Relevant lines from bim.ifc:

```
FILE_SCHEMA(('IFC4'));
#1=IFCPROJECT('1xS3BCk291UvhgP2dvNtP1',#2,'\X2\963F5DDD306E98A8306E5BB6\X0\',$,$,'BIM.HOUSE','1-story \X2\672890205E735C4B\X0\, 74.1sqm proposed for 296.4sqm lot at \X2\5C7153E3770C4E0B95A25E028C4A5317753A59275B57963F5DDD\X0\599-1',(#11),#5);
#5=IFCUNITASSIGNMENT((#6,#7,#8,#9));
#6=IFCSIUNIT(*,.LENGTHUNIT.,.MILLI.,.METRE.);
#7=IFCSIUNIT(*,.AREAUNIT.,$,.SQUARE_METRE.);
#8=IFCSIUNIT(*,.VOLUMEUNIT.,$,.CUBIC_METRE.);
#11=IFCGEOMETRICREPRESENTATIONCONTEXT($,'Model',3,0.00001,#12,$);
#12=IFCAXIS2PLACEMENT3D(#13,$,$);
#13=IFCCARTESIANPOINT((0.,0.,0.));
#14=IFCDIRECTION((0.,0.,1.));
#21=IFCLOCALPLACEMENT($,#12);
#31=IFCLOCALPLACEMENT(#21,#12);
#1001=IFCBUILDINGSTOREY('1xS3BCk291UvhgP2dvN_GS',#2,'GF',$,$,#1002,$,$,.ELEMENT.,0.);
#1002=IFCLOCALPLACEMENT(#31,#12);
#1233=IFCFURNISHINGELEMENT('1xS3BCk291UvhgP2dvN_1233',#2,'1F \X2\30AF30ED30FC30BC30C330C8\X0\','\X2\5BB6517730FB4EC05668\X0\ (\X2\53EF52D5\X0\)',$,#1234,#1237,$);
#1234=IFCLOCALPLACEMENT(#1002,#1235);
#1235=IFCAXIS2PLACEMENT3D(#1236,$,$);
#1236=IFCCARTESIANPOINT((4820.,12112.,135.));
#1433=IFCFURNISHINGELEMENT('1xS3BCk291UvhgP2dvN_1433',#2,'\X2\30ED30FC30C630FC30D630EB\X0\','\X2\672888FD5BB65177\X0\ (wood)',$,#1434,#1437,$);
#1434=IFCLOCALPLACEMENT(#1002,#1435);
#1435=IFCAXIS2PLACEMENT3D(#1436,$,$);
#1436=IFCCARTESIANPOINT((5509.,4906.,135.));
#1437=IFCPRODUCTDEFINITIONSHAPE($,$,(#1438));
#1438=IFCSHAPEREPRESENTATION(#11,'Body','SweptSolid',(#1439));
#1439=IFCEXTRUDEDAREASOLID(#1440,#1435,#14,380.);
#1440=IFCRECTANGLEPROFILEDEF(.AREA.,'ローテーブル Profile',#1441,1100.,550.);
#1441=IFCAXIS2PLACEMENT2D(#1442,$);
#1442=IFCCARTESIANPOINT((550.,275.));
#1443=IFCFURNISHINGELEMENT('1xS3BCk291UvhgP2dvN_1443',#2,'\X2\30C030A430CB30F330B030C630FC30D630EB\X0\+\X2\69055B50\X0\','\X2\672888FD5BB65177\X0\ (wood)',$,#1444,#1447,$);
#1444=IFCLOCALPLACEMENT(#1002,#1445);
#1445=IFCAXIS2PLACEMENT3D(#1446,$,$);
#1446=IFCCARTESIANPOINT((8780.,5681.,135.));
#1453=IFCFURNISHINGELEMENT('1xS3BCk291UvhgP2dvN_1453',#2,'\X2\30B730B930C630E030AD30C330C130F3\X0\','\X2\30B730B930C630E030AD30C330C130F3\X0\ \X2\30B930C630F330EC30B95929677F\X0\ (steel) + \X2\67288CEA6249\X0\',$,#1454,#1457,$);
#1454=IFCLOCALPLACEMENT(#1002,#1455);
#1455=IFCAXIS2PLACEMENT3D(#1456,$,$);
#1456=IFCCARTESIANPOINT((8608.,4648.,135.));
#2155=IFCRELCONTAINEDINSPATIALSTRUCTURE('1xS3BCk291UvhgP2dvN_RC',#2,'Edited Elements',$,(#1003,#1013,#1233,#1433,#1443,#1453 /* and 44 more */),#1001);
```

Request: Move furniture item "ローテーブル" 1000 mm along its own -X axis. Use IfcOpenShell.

```python
import ifcopenshell
import ifcopenshell.api.geometry
import ifcopenshell.util.placement

model = ifcopenshell.open("bim.ifc")

item = model.by_guid("1xS3BCk291UvhgP2dvN_1433")
matrix = ifcopenshell.util.placement.get_local_placement(item.ObjectPlacement)
matrix[:3, 3] -= matrix[:3, 0] * 1000.0
ifcopenshell.api.geometry.edit_object_placement(model, product=item, matrix=matrix, is_si=False)

print(ifcopenshell.util.placement.get_local_placement(item.ObjectPlacement).round(3) + 0.0)

model.write("bim_v2.ifc")
```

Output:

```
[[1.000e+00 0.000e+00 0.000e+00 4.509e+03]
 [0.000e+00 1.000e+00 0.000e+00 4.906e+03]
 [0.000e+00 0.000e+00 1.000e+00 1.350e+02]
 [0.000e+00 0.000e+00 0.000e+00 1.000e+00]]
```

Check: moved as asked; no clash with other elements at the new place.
